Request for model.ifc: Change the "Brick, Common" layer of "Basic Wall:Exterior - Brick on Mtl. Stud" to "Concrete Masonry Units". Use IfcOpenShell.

First a look at what the model holds.

```python
import ifcopenshell
import ifcopenshell.util.element

model = ifcopenshell.open("model.ifc")
print(model.schema)
for layer_set in model.by_type("IfcMaterialLayerSet"):
    if layer_set.LayerSetName == "Basic Wall:Exterior - Brick on Mtl. Stud":
        for layer in layer_set.MaterialLayers:
            print(layer.id(), layer.Material and layer.Material.Name, layer.LayerThickness, sep=" | ")
        print(len(ifcopenshell.util.element.get_elements_by_material(model, layer_set)), "elements and types use it")
print(sorted(m.Name for m in model.by_type("IfcMaterial") if m.Name)[:60])
```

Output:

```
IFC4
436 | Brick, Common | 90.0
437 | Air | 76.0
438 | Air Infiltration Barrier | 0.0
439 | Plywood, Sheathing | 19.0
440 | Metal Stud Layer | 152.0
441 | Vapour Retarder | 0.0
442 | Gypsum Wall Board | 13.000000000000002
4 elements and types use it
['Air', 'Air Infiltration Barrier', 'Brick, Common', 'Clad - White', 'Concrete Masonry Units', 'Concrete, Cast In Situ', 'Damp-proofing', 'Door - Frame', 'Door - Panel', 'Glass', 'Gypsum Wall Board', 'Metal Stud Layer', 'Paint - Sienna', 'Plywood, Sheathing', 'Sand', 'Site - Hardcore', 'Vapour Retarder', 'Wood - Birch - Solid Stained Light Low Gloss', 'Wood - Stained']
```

```python
import ifcopenshell
import ifcopenshell.api.material

model = ifcopenshell.open("model.ifc")

layer_set = next(s for s in model.by_type("IfcMaterialLayerSet") if s.LayerSetName == "Basic Wall:Exterior - Brick on Mtl. Stud")
layer = next(l for l in layer_set.MaterialLayers if l.Material and l.Material.Name == "Brick, Common")
material = next(m for m in model.by_type("IfcMaterial") if m.Name == "Concrete Masonry Units")

# Point this one layer at the other material; renaming the old one would change it everywhere.
ifcopenshell.api.material.edit_layer(model, layer=layer, attributes={"Name": material.Name}, material=material)

print([l.Material.Name if l.Material else None for l in layer_set.MaterialLayers])

model.write("model-out.ifc")
```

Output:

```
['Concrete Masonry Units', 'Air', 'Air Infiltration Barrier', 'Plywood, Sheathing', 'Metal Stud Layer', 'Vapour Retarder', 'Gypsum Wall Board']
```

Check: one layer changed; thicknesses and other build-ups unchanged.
